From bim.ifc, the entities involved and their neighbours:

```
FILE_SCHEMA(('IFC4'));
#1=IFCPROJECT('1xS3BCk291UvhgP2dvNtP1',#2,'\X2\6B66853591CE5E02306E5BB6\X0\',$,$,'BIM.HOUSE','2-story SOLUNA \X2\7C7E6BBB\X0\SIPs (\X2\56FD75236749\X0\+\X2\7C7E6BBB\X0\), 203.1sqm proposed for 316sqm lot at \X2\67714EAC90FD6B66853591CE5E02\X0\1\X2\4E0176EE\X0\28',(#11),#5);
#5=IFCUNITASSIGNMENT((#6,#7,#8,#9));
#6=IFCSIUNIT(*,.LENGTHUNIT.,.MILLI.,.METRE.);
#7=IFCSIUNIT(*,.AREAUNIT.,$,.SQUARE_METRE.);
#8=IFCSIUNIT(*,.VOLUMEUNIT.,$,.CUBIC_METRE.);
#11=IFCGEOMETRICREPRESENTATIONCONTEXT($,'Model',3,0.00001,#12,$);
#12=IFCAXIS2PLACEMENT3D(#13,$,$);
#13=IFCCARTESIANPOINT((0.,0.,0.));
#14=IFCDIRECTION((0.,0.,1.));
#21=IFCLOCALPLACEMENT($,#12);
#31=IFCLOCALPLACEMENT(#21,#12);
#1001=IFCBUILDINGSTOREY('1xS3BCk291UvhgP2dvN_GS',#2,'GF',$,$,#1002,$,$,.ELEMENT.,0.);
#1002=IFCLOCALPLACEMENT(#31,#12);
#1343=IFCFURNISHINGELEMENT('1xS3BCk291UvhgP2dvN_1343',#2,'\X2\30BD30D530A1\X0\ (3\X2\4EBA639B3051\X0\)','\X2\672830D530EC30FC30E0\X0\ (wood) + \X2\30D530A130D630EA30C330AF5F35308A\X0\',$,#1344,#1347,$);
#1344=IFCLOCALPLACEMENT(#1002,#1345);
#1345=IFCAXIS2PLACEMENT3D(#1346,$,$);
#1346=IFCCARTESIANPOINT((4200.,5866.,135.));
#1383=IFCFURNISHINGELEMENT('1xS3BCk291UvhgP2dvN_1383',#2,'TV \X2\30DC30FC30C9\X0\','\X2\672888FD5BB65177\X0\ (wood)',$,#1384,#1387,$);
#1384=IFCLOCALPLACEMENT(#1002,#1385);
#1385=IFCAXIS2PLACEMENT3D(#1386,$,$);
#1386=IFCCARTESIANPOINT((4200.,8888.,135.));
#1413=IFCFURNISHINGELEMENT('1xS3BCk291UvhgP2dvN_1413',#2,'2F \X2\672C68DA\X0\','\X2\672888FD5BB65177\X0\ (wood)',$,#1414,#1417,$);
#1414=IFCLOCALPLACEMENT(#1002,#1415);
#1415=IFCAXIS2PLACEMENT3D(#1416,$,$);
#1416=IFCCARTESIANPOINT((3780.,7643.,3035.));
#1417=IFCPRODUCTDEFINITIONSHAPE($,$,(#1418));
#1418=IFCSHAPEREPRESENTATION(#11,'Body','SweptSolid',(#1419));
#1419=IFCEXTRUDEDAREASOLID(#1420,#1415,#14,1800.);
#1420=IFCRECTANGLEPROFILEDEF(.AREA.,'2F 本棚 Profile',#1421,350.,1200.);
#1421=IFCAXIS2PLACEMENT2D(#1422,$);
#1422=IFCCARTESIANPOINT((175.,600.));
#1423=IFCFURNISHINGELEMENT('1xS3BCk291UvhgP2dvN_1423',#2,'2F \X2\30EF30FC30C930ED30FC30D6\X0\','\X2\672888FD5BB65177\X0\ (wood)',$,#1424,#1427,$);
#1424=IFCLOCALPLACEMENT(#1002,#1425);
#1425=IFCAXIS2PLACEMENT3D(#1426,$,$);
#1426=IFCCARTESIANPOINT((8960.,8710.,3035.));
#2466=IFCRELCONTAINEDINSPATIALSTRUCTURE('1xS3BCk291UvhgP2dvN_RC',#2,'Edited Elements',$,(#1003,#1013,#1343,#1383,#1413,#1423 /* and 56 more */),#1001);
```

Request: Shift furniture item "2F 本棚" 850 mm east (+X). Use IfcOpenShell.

```python
import ifcopenshell
import ifcopenshell.api.geometry
import ifcopenshell.util.placement
import ifcopenshell.util.unit

model = ifcopenshell.open("bim.ifc")
unit_scale = ifcopenshell.util.unit.calculate_unit_scale(model)

item = model.by_id(1413)
matrix = ifcopenshell.util.placement.get_local_placement(item.ObjectPlacement)
matrix[0, 3] += 0.85 / unit_scale
ifcopenshell.api.geometry.edit_object_placement(model, product=item, matrix=matrix, is_si=False)

print(ifcopenshell.util.placement.get_local_placement(item.ObjectPlacement).round(3) + 0.0)

model.write("bim-out.ifc")
```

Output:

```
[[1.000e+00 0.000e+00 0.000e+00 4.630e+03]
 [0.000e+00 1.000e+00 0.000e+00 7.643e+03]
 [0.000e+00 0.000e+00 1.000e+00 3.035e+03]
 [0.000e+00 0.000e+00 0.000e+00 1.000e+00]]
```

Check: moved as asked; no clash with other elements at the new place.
